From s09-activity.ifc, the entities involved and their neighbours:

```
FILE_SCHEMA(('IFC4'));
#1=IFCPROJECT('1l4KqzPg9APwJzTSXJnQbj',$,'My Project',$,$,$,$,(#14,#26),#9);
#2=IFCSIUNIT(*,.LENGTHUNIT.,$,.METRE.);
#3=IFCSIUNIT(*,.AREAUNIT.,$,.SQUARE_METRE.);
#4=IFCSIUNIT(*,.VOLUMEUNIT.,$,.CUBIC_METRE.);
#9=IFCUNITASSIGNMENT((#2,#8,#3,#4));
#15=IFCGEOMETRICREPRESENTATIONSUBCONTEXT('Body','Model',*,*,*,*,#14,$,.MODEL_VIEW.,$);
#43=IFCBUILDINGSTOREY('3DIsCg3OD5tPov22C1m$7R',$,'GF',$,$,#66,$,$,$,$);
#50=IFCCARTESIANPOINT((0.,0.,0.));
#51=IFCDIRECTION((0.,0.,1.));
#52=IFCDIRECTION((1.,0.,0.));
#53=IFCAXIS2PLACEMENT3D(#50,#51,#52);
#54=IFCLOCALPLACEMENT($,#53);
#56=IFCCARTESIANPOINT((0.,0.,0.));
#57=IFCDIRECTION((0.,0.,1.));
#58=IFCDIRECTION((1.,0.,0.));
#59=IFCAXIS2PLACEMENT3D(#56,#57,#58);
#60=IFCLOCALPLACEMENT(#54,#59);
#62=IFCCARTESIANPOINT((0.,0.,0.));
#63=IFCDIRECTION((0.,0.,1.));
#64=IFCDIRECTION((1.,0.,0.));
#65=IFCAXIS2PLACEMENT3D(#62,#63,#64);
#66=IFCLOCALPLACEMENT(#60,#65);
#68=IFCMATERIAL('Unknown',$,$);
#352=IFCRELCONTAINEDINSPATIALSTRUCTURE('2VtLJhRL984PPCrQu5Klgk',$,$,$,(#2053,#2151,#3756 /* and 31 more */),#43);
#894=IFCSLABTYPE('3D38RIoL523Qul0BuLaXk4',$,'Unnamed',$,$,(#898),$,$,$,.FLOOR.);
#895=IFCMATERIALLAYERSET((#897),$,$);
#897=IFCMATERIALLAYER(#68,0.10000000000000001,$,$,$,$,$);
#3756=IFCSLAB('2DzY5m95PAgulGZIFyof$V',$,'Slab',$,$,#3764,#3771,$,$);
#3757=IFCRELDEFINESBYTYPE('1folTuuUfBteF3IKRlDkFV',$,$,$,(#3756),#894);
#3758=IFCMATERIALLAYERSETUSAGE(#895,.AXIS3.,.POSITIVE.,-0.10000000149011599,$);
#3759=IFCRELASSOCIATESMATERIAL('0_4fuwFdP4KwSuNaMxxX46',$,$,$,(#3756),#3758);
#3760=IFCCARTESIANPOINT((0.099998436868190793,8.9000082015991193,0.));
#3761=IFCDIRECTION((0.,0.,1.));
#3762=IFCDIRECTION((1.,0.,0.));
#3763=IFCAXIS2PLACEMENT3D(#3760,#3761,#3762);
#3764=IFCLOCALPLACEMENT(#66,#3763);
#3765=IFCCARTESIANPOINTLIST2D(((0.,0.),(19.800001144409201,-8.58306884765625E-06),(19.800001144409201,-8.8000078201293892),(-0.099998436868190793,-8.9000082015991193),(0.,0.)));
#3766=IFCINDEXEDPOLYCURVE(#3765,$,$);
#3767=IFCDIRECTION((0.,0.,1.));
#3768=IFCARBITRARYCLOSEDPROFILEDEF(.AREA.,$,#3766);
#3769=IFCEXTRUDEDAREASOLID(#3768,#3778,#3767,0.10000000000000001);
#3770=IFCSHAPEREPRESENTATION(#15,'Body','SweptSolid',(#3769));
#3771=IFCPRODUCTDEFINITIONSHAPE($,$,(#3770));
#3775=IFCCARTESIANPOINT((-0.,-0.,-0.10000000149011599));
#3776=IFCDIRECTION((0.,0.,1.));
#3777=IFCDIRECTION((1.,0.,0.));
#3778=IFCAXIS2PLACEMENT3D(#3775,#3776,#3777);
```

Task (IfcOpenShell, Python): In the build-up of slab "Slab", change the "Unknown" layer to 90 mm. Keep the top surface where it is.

```python
import ifcopenshell
import ifcopenshell.util.element
import ifcopenshell.util.representation
import ifcopenshell.util.unit

model = ifcopenshell.open("s09-activity.ifc")
unit_scale = ifcopenshell.util.unit.calculate_unit_scale(model)

layer_set = model.by_id(895)
layer = next(l for l in layer_set.MaterialLayers if l.Material and l.Material.Name == "Unknown")
change = 0.09 / unit_scale - layer.LayerThickness
layer.LayerThickness += change

# Geometry does not follow the layer set by itself.
slabs = [e for e in ifcopenshell.util.element.get_elements_by_material(model, layer_set) if e.is_a("IfcSlab")]
for slab in sorted(slabs, key=lambda e: e.id()):
    body = ifcopenshell.util.representation.get_representation(slab, "Model", "Body")
    solid = body.Items[0]
    old_depth = solid.Depth
    solid.Depth += change
    # Extruded upwards: lower the start of the extrusion so the top stays.
    x, y, z = solid.Position.Location.Coordinates
    solid.Position.Location = model.createIfcCartesianPoint((x, y, z - change))
    print(slab.id(), f"{old_depth:g} -> {solid.Depth:g}")

# The layers are counted up from the underside, which has moved.
for usage in {ifcopenshell.util.element.get_material(slab) for slab in slabs}:
    usage.OffsetFromReferenceLine -= change

model.write("s09-activity_edited.ifc")
```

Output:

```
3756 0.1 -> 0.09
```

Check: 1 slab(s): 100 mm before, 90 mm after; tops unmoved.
